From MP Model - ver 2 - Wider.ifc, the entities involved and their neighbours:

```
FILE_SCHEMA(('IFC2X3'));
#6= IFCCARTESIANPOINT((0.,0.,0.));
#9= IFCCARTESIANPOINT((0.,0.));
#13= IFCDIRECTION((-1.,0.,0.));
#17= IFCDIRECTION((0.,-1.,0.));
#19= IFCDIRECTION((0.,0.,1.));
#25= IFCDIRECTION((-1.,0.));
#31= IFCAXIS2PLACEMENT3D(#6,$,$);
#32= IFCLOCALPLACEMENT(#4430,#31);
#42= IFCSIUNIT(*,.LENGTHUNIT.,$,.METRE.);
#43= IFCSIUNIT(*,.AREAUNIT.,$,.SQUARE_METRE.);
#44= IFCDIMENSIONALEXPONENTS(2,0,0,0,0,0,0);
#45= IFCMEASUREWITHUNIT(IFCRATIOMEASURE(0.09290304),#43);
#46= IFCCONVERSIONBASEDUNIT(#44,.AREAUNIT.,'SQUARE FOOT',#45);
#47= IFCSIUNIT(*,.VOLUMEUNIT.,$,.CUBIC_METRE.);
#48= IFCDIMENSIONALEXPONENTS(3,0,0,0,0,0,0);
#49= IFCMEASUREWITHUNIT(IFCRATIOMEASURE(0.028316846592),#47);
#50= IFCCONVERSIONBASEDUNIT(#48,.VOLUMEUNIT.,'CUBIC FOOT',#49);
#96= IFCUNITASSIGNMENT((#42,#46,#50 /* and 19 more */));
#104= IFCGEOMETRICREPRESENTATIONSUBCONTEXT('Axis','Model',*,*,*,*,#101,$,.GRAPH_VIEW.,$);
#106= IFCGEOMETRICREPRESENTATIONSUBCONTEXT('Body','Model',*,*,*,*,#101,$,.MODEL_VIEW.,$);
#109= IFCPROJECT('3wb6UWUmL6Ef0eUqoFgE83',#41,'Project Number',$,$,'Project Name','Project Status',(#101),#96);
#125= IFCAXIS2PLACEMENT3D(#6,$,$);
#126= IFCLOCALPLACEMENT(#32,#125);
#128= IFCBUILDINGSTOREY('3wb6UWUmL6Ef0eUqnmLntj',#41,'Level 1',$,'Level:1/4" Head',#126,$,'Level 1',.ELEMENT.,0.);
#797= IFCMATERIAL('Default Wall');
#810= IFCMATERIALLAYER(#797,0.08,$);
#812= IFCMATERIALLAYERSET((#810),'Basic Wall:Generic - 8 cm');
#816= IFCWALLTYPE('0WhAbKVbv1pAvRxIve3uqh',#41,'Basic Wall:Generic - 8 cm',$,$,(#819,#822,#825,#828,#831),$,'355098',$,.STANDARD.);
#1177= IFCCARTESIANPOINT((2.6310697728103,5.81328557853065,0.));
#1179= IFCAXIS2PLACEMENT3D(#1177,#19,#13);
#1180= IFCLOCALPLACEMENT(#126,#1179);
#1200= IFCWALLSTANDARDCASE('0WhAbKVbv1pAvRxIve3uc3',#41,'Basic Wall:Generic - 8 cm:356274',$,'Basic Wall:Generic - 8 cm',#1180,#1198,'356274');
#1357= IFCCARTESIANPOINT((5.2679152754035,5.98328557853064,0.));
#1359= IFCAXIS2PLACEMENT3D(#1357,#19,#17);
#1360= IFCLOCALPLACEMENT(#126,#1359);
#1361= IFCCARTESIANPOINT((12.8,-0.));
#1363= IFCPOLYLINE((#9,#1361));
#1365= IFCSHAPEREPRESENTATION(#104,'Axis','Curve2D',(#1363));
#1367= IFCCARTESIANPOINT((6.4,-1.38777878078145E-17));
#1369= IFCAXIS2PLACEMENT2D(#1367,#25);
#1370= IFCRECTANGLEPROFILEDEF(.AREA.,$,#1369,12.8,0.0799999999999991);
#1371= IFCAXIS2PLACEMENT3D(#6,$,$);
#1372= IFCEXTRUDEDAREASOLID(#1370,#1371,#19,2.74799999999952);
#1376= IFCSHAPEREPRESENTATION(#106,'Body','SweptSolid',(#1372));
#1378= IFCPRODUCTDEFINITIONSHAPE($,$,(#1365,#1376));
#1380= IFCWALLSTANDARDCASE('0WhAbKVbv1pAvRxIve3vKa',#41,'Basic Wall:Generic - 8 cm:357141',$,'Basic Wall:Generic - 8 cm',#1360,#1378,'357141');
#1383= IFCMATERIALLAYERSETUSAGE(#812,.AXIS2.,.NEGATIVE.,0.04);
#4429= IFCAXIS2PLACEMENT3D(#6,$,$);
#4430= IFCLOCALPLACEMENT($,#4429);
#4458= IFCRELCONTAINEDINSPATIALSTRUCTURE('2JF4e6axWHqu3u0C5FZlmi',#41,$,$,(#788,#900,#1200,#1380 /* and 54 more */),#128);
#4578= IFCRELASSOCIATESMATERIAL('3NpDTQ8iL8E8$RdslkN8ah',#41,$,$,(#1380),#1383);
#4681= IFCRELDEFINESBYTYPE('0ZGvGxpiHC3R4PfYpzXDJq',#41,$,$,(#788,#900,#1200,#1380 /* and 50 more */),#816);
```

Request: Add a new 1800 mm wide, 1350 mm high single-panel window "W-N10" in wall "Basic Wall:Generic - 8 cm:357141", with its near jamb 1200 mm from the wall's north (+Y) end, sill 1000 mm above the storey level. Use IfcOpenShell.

```python
import numpy as np
import ifcopenshell
import ifcopenshell.api.feature
import ifcopenshell.api.geometry
import ifcopenshell.api.root
import ifcopenshell.api.spatial
import ifcopenshell.api.type
import ifcopenshell.geom
import ifcopenshell.util.element
import ifcopenshell.util.placement
import ifcopenshell.util.representation
import ifcopenshell.util.shape
import ifcopenshell.util.unit

model = ifcopenshell.open("MP Model - ver 2 - Wider.ifc")
unit_scale = ifcopenshell.util.unit.calculate_unit_scale(model)
settings = ifcopenshell.geom.settings()


def volume(element):
    """Net volume in cubic metres, openings subtracted."""
    shape = ifcopenshell.geom.create_shape(settings, element)
    return ifcopenshell.util.shape.get_volume(shape.geometry)


wall = model.by_id(1380)
storey = ifcopenshell.util.element.get_container(wall, ifc_class="IfcBuildingStorey")
context = ifcopenshell.util.representation.get_context(model, "Model", "Body", "MODEL_VIEW")
before = volume(wall)

width, height, from_end, sill = 1.8, 1.35, 1.2, 1  # metres

# The wall runs along its own X axis, and the end named is its -X end.
wall_shape = ifcopenshell.geom.create_shape(settings, wall)
x, y, z = ifcopenshell.util.shape.get_vertices(wall_shape.geometry).T
start = x.min() + from_end
face, thickness = float(y.min()), float(y.max() - y.min())
wall_matrix = ifcopenshell.util.placement.get_local_placement(wall.ObjectPlacement)
level = ifcopenshell.util.placement.get_local_placement(storey.ObjectPlacement)[2, 3]


def in_wall(x, y):
    """Placement at x, y metres in the wall's axes, at sill height."""
    matrix = wall_matrix.copy()
    matrix[:, 3] = wall_matrix @ np.array([x / unit_scale, y / unit_scale, 0.0, 1.0])
    matrix[2, 3] = level + sill / unit_scale
    return matrix


# Opening: a box that overshoots both wall faces by 50 mm.
opening = ifcopenshell.api.root.create_entity(model, ifc_class="IfcOpeningElement")
box = ifcopenshell.api.geometry.add_wall_representation(
    model, context=context, length=width, height=height, thickness=thickness + 0.1
)
ifcopenshell.api.geometry.assign_representation(model, product=opening, representation=box)
ifcopenshell.api.geometry.edit_object_placement(model, product=opening, matrix=in_wall(start, face - 0.05), is_si=False)
ifcopenshell.api.feature.add_feature(model, feature=opening, element=wall)

window = ifcopenshell.api.root.create_entity(model, ifc_class="IfcWindow", name="W-N10")
window.OverallWidth, window.OverallHeight = width / unit_scale, height / unit_scale
body = ifcopenshell.api.geometry.add_window_representation(
    model,
    context=context,
    overall_width=window.OverallWidth,
    overall_height=window.OverallHeight,
    partition_type="SINGLE_PANEL",
)
ifcopenshell.api.geometry.assign_representation(model, product=window, representation=body)
ifcopenshell.api.spatial.assign_container(model, products=[window], relating_structure=storey)
fills = ifcopenshell.api.feature.add_filling(model, opening=opening, element=window)
fills.OwnerHistory = window.OwnerHistory  # required in IFC2X3

# IFC2X3 keeps the operation on the window style.
style = ifcopenshell.api.root.create_entity(model, ifc_class="IfcWindowStyle", name="W-N10")
style.OperationType, style.ConstructionType = "SINGLE_PANEL", "NOTDEFINED"
style.ParameterTakesPrecedence = style.Sizeable = False
ifcopenshell.api.type.assign_type(model, related_objects=[window], relating_type=style)

# Centre the window in the wall's thickness.
ifcopenshell.api.geometry.edit_object_placement(model, product=window, matrix=in_wall(start, face), is_si=False)
window_shape = ifcopenshell.geom.create_shape(settings, window)
depth = ifcopenshell.util.shape.get_vertices(window_shape.geometry)[:, 1]
offset = face + thickness / 2 - (depth.min() + depth.max()) / 2
ifcopenshell.api.geometry.edit_object_placement(model, product=window, matrix=in_wall(start, offset), is_si=False)

after = volume(wall)

print(f"wall volume {before:.3f} -> {after:.3f} m3")

model.write("MP Model - ver 2 - Wider_v2.ifc")
```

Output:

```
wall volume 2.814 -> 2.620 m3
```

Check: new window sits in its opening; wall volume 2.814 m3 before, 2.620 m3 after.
